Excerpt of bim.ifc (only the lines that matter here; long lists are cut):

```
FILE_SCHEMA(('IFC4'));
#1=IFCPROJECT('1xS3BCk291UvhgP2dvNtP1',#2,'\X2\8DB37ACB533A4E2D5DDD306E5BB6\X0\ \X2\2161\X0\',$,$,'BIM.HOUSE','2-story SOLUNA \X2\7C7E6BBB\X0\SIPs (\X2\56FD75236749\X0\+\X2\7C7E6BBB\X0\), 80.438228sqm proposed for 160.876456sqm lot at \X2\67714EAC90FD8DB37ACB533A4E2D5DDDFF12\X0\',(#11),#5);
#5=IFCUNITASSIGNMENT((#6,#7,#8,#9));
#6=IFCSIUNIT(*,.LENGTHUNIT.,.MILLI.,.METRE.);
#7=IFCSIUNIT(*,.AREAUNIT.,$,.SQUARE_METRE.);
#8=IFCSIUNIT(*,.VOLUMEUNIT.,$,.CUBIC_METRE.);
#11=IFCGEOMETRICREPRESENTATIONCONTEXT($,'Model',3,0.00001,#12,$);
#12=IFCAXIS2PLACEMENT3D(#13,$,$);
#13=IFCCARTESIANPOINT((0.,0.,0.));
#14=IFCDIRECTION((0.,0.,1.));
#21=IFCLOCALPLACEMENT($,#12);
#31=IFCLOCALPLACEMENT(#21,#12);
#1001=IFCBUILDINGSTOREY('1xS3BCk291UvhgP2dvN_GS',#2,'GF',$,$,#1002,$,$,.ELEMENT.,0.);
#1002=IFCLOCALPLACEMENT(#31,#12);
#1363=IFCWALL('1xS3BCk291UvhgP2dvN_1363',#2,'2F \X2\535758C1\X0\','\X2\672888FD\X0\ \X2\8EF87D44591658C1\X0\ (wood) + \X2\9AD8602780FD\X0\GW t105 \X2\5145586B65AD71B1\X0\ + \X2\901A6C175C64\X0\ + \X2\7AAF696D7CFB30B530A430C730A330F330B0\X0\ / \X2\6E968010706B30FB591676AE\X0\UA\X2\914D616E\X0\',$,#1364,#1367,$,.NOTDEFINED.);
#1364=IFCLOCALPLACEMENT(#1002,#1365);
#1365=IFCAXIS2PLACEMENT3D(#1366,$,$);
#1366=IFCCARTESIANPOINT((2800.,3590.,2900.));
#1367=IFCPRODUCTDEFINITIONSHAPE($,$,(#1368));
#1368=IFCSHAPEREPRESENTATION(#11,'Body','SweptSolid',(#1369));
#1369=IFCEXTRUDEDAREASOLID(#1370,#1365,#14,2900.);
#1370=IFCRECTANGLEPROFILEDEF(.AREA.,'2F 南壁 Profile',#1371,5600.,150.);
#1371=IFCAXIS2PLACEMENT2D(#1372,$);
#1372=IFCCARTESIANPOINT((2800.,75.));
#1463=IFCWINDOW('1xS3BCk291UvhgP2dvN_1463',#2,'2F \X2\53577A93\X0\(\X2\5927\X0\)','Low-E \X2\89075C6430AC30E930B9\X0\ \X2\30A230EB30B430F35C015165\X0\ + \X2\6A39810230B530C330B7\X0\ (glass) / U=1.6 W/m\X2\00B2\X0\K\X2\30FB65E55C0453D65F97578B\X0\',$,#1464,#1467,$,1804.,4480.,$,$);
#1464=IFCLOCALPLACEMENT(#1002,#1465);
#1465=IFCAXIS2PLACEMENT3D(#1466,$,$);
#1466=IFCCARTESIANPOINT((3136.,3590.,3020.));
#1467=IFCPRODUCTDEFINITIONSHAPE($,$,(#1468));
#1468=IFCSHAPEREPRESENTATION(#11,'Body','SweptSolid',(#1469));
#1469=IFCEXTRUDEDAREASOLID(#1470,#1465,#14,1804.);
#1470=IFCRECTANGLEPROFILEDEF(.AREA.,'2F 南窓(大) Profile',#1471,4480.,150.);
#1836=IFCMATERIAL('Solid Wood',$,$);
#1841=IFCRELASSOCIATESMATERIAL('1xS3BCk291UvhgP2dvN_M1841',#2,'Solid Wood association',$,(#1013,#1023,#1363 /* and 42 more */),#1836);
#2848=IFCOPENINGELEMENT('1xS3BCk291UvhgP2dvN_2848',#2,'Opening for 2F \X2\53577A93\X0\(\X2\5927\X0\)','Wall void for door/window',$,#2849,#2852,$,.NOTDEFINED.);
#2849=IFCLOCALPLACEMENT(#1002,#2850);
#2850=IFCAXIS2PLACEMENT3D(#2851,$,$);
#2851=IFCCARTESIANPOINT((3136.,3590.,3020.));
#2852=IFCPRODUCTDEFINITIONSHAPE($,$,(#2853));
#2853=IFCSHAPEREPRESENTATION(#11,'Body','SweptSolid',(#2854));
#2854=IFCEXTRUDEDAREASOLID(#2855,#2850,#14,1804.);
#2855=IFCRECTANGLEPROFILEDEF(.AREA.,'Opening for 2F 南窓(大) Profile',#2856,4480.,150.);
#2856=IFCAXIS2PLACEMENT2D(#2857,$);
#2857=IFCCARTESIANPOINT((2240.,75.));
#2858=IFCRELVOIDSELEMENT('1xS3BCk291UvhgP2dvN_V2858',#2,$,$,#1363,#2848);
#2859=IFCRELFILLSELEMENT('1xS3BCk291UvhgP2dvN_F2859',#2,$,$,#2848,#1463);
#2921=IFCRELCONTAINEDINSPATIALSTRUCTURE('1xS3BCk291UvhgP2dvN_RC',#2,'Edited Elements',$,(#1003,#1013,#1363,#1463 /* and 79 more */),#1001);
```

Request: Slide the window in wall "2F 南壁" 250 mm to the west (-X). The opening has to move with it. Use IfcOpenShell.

```python
import ifcopenshell
import ifcopenshell.api.geometry
import ifcopenshell.util.placement

model = ifcopenshell.open("bim.ifc")

window = model.by_id(1463)
opening = window.FillsVoids[0].RelatingOpeningElement
wall = opening.VoidsElements[0].RelatingBuildingElement

wall_matrix = ifcopenshell.util.placement.get_local_placement(wall.ObjectPlacement)
shift = wall_matrix[:3, 0] * -250.0
before = ifcopenshell.util.placement.get_local_placement(window.ObjectPlacement)[:3, 3].copy()

# The window is not placed relative to its opening, so move both.
for product in (opening, window):
    matrix = ifcopenshell.util.placement.get_local_placement(product.ObjectPlacement)
    matrix[:3, 3] += shift
    ifcopenshell.api.geometry.edit_object_placement(model, product=product, matrix=matrix, is_si=False)

after = ifcopenshell.util.placement.get_local_placement(window.ObjectPlacement)[:3, 3]
print("window moved by", (after - before).round(3) + 0.0)

model.write("bim_edited.ifc")
```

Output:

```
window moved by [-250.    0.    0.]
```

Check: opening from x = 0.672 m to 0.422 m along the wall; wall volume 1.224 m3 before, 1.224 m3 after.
